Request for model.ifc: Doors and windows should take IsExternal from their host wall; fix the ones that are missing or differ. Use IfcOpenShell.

First a look at what the model holds.

```python
import ifcopenshell
import ifcopenshell.util.element

model = ifcopenshell.open("model.ifc")
print(model.schema)
seen = {}
for e in model.by_type("IfcDoor") + model.by_type("IfcWindow"):
    if not e.FillsVoids:
        continue
    host = e.FillsVoids[0].RelatingOpeningElement.VoidsElements[0].RelatingBuildingElement
    own = ifcopenshell.util.element.get_pset(e, f"Pset_{e.is_a()[3:].removesuffix('StandardCase')}Common", "IsExternal")
    wall = ifcopenshell.util.element.get_pset(host, "Pset_WallCommon", "IsExternal")
    seen[e.is_a(), own, wall] = seen.get((e.is_a(), own, wall), 0) + 1
for (cls, own, wall), count in sorted(seen.items(), key=str):
    print(count, cls, "IsExternal:", own, "| host wall:", wall)
```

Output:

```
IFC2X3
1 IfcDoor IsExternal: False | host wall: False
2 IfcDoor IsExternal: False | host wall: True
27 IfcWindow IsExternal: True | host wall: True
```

```python
import ifcopenshell
import ifcopenshell.api.pset
import ifcopenshell.util.element

model = ifcopenshell.open("model.ifc")

count = 0
for ifc_class, pset_name in (("IfcDoor", "Pset_DoorCommon"), ("IfcWindow", "Pset_WindowCommon")):
    for e in model.by_type(ifc_class):
        if not e.FillsVoids:
            continue
        host = e.FillsVoids[0].RelatingOpeningElement.VoidsElements[0].RelatingBuildingElement
        external = ifcopenshell.util.element.get_pset(host, "Pset_WallCommon", "IsExternal")
        if external is None or ifcopenshell.util.element.get_pset(e, pset_name, "IsExternal") == external:
            continue
        pset = ifcopenshell.api.pset.add_pset(model, product=e, name=pset_name)
        ifcopenshell.api.pset.edit_pset(model, pset=pset, properties={"IsExternal": external})
        count += 1

print(count, "updated")

model.write("model_v2.ifc")
```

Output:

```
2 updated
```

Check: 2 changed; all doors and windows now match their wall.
